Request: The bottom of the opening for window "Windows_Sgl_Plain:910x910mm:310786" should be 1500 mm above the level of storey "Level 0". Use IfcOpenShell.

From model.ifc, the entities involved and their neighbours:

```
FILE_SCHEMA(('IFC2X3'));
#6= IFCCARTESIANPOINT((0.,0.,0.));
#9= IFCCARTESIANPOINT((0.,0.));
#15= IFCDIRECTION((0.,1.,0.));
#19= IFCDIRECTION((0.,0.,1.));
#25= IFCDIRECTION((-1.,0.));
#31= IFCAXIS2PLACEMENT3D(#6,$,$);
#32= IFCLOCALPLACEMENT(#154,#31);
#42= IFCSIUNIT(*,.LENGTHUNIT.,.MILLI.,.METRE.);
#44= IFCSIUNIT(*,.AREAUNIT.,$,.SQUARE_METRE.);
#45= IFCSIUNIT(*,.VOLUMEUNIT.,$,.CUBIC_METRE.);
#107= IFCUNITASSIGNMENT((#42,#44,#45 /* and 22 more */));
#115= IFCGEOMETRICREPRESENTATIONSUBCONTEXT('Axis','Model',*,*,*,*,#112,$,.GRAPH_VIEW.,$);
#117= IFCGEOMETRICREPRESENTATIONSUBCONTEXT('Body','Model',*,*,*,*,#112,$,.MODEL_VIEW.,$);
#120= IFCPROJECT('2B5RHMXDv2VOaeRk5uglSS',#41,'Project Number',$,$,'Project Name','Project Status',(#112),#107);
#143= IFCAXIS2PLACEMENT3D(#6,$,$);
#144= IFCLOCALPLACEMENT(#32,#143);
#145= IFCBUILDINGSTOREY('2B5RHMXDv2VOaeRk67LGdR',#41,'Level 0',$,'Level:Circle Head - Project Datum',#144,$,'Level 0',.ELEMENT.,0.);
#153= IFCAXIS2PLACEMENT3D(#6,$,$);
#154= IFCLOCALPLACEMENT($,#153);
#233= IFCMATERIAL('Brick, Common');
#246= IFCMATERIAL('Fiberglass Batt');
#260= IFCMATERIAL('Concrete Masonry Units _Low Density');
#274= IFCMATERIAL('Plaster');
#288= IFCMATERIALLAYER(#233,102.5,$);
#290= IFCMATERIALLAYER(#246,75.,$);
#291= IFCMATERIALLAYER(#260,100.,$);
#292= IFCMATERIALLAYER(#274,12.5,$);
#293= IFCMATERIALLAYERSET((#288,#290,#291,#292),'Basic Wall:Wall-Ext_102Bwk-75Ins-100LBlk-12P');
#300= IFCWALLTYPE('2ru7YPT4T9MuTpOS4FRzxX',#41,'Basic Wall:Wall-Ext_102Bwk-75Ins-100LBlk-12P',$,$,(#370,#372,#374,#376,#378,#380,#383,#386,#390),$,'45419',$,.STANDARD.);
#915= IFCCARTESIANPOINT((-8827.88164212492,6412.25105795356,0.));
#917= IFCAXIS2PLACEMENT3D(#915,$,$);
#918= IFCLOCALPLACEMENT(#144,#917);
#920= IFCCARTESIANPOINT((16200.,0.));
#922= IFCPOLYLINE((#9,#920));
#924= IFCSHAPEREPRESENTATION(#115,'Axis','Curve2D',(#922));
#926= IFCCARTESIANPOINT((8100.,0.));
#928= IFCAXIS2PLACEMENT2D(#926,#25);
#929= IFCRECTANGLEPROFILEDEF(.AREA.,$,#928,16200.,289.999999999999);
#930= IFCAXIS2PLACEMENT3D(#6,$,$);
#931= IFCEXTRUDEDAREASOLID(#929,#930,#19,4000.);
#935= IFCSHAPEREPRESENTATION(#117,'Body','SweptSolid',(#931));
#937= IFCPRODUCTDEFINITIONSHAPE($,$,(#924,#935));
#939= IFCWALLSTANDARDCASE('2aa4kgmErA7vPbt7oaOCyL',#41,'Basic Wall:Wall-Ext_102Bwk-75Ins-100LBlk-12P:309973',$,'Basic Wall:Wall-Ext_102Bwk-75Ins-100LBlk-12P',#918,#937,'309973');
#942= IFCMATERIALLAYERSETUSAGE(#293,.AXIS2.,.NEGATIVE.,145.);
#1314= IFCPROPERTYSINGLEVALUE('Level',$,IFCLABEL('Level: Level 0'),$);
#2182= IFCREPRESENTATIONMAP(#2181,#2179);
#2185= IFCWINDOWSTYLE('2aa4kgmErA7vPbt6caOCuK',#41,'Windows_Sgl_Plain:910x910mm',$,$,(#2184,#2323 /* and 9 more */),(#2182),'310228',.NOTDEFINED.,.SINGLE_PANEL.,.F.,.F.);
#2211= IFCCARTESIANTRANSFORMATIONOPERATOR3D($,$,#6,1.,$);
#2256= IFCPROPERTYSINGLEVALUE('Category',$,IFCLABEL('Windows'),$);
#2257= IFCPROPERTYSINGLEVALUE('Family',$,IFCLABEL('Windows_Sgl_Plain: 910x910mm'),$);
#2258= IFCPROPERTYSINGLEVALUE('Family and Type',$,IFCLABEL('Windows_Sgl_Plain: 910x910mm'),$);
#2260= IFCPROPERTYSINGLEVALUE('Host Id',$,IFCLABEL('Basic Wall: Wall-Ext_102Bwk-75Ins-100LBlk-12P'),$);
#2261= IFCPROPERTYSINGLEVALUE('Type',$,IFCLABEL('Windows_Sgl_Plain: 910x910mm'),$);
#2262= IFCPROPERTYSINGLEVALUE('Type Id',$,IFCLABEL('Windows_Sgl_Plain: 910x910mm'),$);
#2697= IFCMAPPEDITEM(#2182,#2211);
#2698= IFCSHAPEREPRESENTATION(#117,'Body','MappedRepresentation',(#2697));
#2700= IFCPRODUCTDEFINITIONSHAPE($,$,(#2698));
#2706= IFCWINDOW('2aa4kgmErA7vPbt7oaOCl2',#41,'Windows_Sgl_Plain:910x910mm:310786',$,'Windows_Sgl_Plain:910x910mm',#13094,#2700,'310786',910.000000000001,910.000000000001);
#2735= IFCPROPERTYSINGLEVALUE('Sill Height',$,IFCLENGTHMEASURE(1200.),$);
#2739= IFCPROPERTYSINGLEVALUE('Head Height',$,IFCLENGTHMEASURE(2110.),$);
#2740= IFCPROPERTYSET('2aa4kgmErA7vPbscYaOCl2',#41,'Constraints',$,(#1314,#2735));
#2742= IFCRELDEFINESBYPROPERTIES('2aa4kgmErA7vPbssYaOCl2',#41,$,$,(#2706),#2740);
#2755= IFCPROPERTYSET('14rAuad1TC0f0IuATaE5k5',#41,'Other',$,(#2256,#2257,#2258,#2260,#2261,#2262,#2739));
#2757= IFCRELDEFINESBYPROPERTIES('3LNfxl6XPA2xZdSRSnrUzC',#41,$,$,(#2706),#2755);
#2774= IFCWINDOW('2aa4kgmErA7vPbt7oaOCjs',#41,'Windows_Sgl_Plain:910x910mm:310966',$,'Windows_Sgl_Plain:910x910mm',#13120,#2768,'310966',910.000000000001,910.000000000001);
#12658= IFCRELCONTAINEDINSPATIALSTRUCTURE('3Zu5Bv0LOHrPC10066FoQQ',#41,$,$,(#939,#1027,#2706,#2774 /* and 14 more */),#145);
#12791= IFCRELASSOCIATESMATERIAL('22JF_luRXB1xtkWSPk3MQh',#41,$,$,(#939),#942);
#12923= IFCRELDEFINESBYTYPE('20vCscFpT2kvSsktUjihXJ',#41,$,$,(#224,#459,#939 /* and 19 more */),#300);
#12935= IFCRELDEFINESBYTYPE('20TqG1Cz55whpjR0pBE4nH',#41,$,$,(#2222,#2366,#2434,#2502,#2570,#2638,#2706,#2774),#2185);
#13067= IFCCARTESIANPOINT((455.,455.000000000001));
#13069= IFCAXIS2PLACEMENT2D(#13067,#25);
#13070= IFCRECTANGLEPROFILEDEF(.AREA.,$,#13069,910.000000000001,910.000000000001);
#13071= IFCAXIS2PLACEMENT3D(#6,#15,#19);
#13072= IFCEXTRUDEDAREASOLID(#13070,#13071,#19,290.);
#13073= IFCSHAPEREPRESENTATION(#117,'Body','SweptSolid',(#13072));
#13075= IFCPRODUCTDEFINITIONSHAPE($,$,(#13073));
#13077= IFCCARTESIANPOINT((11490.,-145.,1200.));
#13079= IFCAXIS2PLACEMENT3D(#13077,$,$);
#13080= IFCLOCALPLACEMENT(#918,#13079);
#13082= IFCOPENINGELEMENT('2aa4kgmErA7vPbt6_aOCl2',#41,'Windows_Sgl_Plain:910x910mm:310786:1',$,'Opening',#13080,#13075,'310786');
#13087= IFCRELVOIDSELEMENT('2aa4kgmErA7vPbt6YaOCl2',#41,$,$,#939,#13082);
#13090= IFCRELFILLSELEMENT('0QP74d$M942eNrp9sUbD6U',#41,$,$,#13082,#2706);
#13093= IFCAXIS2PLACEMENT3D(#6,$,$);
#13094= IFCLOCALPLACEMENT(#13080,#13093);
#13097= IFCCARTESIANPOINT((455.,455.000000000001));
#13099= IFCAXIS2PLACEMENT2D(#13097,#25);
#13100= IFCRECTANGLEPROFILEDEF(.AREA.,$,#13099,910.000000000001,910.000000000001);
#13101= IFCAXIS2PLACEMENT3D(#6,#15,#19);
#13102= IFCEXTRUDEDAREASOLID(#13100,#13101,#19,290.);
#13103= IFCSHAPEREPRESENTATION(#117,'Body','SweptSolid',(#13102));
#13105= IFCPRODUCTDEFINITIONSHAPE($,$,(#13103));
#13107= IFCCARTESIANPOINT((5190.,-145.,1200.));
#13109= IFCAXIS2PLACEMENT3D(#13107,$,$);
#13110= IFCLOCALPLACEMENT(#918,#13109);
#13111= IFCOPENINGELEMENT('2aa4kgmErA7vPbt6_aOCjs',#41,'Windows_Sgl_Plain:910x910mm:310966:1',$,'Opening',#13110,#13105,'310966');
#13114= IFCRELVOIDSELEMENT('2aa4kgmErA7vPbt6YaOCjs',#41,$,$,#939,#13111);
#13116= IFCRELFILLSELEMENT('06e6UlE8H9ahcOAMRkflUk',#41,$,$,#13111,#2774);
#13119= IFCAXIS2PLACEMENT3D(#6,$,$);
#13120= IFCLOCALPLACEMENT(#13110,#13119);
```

```python
import numpy as np
import ifcopenshell
import ifcopenshell.api.geometry
import ifcopenshell.api.pset
import ifcopenshell.geom
import ifcopenshell.util.element
import ifcopenshell.util.placement
import ifcopenshell.util.shape
import ifcopenshell.util.unit

model = ifcopenshell.open("model.ifc")
unit_scale = ifcopenshell.util.unit.calculate_unit_scale(model)

window = model.by_guid("2aa4kgmErA7vPbt7oaOCl2")
opening = window.FillsVoids[0].RelatingOpeningElement
storey = ifcopenshell.util.element.get_container(window, ifc_class="IfcBuildingStorey")
level = ifcopenshell.util.placement.get_local_placement(storey.ObjectPlacement)[2, 3]

# The opening's origin need not be at the sill, so measure its lowest point.
shape = ifcopenshell.geom.create_shape(ifcopenshell.geom.settings(), opening)
bottom = ifcopenshell.util.shape.get_shape_bottom_elevation(shape, shape.geometry) / unit_scale
dz = level + 1.5 / unit_scale - bottom

shift = np.array([0.0, 0.0, dz])
# The window is placed relative to its opening, so it follows when the opening moves.
matrix = ifcopenshell.util.placement.get_local_placement(opening.ObjectPlacement)
matrix[:3, 3] += shift
ifcopenshell.api.geometry.edit_object_placement(
    model, product=opening, matrix=matrix, is_si=False, should_transform_children=True
)

# Keep the stored heights in step.
pset = model.by_id(ifcopenshell.util.element.get_pset(window, "Constraints", should_inherit=False)["id"])
ifcopenshell.api.pset.edit_pset(model, pset=pset, properties={
    "Sill Height": model.create_entity("IfcLengthMeasure", ifcopenshell.util.element.get_pset(window, "Constraints", "Sill Height") + dz),
})
pset = model.by_id(ifcopenshell.util.element.get_pset(window, "Other", should_inherit=False)["id"])
ifcopenshell.api.pset.edit_pset(model, pset=pset, properties={
    "Head Height": model.create_entity("IfcLengthMeasure", ifcopenshell.util.element.get_pset(window, "Other", "Head Height") + dz),
})

print(f"moved by {dz * unit_scale:+.3f} m")

model.write("model_updated.ifc")
```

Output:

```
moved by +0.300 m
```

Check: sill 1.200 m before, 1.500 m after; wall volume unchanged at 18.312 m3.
